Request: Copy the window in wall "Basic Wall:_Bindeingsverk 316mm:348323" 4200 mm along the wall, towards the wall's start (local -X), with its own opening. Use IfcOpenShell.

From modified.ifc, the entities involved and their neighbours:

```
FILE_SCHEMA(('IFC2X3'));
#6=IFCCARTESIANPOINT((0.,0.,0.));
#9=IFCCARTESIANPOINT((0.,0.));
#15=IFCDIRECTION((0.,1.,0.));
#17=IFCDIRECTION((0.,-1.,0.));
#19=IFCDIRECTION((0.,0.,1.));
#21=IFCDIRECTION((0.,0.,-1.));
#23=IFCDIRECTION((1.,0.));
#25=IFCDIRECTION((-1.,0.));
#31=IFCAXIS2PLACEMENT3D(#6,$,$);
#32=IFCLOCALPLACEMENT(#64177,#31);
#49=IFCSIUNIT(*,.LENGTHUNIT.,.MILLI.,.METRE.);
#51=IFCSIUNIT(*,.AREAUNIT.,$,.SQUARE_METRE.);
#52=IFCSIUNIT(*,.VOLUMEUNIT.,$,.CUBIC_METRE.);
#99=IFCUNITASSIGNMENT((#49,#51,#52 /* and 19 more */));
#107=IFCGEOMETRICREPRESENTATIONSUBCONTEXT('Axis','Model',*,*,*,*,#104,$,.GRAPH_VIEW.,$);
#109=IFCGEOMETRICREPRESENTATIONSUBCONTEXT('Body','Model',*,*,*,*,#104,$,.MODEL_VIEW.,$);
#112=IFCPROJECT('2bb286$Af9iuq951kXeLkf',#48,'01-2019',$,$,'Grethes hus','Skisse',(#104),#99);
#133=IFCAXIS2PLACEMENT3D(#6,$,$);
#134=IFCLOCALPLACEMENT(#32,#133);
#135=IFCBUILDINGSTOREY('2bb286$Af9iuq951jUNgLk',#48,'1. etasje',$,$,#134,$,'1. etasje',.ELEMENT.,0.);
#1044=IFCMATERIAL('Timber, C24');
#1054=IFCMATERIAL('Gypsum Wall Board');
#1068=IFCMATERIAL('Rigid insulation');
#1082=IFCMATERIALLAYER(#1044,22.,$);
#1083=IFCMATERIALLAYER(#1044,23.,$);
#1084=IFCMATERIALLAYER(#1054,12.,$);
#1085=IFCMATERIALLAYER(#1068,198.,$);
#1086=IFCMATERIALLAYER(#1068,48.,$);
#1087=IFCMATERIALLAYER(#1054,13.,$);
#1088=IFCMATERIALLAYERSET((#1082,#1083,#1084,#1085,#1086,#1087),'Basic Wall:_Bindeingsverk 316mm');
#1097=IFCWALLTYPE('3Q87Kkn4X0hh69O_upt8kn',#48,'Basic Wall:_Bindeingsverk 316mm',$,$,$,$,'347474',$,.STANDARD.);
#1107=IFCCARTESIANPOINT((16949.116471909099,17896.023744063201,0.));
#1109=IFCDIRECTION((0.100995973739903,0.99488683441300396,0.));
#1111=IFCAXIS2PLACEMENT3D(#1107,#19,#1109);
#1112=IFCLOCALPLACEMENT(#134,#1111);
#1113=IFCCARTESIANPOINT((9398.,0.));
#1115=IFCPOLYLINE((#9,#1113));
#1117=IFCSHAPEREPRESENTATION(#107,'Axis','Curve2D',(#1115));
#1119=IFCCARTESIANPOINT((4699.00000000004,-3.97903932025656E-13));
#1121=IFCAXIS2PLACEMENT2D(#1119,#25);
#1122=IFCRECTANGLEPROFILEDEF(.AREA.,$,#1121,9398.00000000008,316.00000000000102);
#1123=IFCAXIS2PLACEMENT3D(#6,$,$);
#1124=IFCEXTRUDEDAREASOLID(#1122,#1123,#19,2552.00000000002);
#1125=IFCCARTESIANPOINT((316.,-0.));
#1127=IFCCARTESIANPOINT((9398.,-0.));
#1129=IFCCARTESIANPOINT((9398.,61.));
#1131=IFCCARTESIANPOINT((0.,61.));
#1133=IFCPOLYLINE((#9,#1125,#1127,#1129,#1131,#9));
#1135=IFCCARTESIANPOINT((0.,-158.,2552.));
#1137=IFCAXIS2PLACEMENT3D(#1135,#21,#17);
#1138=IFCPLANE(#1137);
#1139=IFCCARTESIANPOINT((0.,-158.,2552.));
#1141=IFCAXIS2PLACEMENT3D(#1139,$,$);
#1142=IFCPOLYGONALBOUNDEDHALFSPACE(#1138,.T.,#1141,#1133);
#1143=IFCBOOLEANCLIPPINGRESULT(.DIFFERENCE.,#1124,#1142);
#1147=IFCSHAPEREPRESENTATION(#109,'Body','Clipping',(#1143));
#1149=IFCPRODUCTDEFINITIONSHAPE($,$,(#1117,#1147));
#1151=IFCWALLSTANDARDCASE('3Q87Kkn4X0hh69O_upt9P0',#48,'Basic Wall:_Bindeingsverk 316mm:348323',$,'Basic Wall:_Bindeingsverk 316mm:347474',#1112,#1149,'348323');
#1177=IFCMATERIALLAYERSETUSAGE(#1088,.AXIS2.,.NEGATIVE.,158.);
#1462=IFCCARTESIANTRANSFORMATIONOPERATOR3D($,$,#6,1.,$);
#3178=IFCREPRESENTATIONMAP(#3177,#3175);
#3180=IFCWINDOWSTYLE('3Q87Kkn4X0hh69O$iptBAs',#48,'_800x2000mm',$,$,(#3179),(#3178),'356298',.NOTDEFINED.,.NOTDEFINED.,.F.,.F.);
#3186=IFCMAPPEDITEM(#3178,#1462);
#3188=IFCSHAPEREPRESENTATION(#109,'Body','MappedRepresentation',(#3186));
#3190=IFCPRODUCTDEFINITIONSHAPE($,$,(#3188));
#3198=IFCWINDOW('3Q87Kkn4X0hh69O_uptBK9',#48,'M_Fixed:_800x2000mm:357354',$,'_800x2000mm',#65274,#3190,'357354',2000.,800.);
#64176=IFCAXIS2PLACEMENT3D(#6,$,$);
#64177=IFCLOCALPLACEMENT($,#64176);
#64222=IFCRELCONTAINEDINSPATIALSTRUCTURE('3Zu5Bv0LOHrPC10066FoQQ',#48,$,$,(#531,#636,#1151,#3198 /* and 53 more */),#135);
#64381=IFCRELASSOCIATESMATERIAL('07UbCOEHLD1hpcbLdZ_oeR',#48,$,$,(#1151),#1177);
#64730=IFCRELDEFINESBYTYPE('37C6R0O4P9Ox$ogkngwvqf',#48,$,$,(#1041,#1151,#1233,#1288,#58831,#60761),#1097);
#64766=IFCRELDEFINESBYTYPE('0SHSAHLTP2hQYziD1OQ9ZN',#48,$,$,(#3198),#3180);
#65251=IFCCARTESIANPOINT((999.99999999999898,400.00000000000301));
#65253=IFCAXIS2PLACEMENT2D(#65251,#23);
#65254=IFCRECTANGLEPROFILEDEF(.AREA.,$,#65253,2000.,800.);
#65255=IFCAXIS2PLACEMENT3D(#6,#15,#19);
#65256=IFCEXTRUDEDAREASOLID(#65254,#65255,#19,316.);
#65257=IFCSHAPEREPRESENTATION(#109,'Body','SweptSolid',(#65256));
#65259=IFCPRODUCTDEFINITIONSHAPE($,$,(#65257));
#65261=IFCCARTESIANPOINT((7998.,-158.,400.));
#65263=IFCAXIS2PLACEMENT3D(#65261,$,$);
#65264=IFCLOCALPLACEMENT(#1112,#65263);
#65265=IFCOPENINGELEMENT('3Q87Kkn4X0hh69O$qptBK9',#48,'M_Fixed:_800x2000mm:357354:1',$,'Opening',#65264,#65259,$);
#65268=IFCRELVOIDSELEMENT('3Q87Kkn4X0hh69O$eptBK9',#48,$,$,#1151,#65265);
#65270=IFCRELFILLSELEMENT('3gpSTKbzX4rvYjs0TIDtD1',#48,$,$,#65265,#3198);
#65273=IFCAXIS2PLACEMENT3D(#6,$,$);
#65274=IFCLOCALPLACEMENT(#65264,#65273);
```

```python
import ifcopenshell
import ifcopenshell.api.feature
import ifcopenshell.api.geometry
import ifcopenshell.api.root
import ifcopenshell.geom
import ifcopenshell.util.element
import ifcopenshell.util.placement
import ifcopenshell.util.shape
import ifcopenshell.util.unit

model = ifcopenshell.open("modified.ifc")
unit_scale = ifcopenshell.util.unit.calculate_unit_scale(model)
settings = ifcopenshell.geom.settings()


def volume(element):
    """Net volume in cubic metres, openings subtracted."""
    shape = ifcopenshell.geom.create_shape(settings, element)
    return ifcopenshell.util.shape.get_volume(shape.geometry)


def reuse_history(source, copy):
    """copy_class also copies each property set's owner history, people and application; keep the originals."""
    for rel in copy.IsDefinedBy:
        if rel.is_a("IfcRelDefinesByProperties") and (history := rel.RelatingPropertyDefinition.OwnerHistory):
            rel.RelatingPropertyDefinition.OwnerHistory = source.OwnerHistory
            ifcopenshell.util.element.remove_deep2(model, history)


window = model.by_id(3198)
opening = window.FillsVoids[0].RelatingOpeningElement
wall = opening.VoidsElements[0].RelatingBuildingElement
before = volume(wall)
shift = ifcopenshell.util.placement.get_local_placement(wall.ObjectPlacement)[:3, 0] * -4.2 / unit_scale

# copy_class copies the void relationship, type, container and properties, but no geometry.
new_opening = ifcopenshell.api.root.copy_class(model, product=opening)
new_opening.Representation = ifcopenshell.util.element.copy_deep(
    model, opening.Representation, exclude=["IfcGeometricRepresentationContext", "IfcRepresentationMap"]
)
new_opening.Name = "M_Fixed:_800x2000mm"
new_window = ifcopenshell.api.root.copy_class(model, product=window)
new_window.Representation = ifcopenshell.util.element.copy_deep(
    model, window.Representation, exclude=["IfcGeometricRepresentationContext", "IfcRepresentationMap"]
)
new_window.Name = "M_Fixed:_800x2000mm"
new_window.Tag = None
reuse_history(window, new_window)
fills = ifcopenshell.api.feature.add_filling(model, opening=new_opening, element=new_window)
fills.OwnerHistory = new_window.OwnerHistory  # required in IFC2X3

for old, new in ((opening, new_opening), (window, new_window)):
    matrix = ifcopenshell.util.placement.get_local_placement(old.ObjectPlacement)
    matrix[:3, 3] += shift
    ifcopenshell.api.geometry.edit_object_placement(model, product=new, matrix=matrix, is_si=False)

after = volume(wall)

print(f"wall volume {before:.3f} -> {after:.3f} m3")

model.write("modified_v2.ifc")
```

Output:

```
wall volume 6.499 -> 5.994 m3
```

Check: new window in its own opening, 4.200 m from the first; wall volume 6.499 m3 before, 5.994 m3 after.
